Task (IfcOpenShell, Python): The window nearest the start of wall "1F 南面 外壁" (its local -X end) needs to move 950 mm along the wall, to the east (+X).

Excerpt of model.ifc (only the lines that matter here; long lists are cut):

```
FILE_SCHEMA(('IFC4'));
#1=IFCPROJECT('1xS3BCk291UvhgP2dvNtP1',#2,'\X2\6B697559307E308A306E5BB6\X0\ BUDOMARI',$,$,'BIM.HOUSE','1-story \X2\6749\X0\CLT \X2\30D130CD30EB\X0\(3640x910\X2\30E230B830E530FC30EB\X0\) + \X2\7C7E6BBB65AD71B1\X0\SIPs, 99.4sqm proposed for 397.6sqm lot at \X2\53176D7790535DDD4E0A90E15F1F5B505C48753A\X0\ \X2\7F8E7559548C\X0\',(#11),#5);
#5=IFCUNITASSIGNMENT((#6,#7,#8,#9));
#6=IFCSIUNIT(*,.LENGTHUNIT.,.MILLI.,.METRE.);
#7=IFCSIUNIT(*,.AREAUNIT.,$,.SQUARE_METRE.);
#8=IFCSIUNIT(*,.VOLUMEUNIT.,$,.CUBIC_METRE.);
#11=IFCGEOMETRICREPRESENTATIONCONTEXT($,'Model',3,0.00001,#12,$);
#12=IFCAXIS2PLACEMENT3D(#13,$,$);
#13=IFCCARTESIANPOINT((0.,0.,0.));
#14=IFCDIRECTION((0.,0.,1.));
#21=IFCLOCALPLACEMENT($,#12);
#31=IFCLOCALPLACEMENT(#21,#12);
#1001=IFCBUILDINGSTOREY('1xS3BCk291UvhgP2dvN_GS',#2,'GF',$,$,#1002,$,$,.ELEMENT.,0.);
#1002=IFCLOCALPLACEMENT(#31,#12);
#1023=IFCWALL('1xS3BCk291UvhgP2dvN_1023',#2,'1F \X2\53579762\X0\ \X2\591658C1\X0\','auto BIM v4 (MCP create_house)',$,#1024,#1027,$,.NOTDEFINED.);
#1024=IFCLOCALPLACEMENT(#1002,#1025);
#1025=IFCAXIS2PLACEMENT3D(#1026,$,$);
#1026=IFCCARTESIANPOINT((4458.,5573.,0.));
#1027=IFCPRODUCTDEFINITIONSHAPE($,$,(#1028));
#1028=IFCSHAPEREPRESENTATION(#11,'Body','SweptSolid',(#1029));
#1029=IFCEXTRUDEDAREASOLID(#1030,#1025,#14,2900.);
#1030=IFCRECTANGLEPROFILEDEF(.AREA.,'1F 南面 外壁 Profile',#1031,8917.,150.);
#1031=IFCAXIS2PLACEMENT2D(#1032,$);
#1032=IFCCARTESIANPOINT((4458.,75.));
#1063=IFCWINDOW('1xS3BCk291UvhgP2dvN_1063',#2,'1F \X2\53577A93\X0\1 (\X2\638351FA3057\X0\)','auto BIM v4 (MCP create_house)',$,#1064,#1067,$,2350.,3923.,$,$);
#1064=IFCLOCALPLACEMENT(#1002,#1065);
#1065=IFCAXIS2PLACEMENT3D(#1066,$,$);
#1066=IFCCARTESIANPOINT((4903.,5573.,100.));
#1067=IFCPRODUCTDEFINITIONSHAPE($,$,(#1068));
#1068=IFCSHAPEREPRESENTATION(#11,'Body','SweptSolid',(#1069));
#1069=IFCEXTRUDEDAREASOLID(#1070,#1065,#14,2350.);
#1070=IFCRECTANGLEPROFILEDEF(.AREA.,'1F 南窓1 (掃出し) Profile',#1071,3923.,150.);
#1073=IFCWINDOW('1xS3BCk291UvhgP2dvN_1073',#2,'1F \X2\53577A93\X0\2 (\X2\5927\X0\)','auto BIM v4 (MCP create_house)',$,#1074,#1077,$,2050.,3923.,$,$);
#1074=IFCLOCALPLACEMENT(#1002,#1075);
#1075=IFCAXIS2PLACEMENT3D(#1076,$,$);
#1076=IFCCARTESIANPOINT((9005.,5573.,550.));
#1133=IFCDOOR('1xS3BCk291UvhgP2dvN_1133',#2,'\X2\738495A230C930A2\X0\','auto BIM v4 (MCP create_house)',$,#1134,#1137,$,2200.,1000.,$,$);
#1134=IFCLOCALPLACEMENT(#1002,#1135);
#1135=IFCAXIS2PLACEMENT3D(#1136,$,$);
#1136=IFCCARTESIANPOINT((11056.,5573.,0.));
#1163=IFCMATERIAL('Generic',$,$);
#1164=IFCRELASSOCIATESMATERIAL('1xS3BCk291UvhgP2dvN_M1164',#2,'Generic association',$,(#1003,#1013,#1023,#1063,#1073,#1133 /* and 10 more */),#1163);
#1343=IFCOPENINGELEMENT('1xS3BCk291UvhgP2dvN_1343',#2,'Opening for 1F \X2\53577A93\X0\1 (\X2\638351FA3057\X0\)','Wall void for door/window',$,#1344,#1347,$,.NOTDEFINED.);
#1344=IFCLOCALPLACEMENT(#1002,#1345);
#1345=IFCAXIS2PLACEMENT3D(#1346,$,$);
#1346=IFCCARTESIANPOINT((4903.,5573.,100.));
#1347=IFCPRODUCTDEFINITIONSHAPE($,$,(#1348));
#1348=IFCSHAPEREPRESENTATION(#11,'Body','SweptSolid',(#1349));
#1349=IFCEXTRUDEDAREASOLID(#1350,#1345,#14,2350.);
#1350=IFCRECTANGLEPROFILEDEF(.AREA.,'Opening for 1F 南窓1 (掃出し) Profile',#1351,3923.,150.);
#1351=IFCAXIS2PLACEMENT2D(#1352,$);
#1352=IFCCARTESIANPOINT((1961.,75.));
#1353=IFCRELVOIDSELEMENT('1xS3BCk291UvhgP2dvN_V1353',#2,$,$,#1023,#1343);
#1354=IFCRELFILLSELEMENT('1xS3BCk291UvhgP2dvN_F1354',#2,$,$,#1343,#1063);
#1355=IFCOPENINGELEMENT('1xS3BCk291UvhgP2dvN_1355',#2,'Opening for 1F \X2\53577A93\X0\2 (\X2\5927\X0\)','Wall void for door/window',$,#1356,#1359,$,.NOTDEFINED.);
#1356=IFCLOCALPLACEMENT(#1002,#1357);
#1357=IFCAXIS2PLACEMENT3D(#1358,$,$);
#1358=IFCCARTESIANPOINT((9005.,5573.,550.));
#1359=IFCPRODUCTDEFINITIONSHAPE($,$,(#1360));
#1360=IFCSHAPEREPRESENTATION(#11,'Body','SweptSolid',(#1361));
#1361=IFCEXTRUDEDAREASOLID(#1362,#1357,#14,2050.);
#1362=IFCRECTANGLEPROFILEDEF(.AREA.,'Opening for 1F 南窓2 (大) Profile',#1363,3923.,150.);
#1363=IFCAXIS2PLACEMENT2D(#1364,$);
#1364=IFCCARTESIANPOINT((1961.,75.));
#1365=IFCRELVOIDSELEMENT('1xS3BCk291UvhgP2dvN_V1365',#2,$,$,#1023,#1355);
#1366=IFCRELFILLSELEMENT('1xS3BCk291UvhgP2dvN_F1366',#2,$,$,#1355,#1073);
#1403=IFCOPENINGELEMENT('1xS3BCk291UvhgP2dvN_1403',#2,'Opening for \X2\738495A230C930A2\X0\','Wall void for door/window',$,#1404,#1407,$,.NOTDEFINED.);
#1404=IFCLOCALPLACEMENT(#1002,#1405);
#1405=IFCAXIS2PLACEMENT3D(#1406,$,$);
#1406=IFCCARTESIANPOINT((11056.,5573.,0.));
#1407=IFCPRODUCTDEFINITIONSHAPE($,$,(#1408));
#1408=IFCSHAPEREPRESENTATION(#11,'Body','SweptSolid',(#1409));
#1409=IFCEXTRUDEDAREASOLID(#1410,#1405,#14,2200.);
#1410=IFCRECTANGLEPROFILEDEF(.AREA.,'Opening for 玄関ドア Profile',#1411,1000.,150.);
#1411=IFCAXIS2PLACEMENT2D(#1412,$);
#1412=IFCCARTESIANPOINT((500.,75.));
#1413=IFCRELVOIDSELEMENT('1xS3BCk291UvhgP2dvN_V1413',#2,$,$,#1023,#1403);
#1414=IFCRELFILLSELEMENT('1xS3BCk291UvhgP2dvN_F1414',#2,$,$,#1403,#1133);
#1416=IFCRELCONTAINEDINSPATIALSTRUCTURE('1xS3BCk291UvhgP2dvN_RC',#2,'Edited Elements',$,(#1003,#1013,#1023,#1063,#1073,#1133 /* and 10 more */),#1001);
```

```python
import ifcopenshell
import ifcopenshell.api.geometry
import ifcopenshell.util.placement
import ifcopenshell.util.unit

model = ifcopenshell.open("model.ifc")
unit_scale = ifcopenshell.util.unit.calculate_unit_scale(model)

window = model.by_guid("1xS3BCk291UvhgP2dvN_1063")
opening = window.FillsVoids[0].RelatingOpeningElement
wall = opening.VoidsElements[0].RelatingBuildingElement

wall_matrix = ifcopenshell.util.placement.get_local_placement(wall.ObjectPlacement)
shift = wall_matrix[:3, 0] * 0.95 / unit_scale
before = ifcopenshell.util.placement.get_local_placement(window.ObjectPlacement)[:3, 3].copy()

# The window is not placed relative to its opening, so move both.
for product in (opening, window):
    matrix = ifcopenshell.util.placement.get_local_placement(product.ObjectPlacement)
    matrix[:3, 3] += shift
    ifcopenshell.api.geometry.edit_object_placement(model, product=product, matrix=matrix, is_si=False)

after = ifcopenshell.util.placement.get_local_placement(window.ObjectPlacement)[:3, 3]
print("window moved by", (after - before).round(3) + 0.0)

model.write("model_rev.ifc")
```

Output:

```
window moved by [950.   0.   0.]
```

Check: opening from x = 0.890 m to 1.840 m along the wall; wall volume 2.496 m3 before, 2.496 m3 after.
